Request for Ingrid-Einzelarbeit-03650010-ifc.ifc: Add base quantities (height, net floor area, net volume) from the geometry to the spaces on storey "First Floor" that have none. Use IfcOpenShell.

First a look at what the model holds.

```python
import ifcopenshell
import ifcopenshell.util.element
import ifcopenshell.util.unit

model = ifcopenshell.open("Ingrid-Einzelarbeit-03650010-ifc.ifc")
print(model.schema)
for unit_type in ("LENGTHUNIT", "AREAUNIT", "VOLUMEUNIT"):
    print(unit_type, ifcopenshell.util.unit.calculate_unit_scale(model, unit_type))
storey = next(s for s in model.by_type("IfcBuildingStorey") if s.Name == "First Floor")
spaces = [e for e in ifcopenshell.util.element.get_decomposition(storey) if e.is_a("IfcSpace")]
for e in sorted(spaces, key=lambda e: e.id()):
    print(e.id(), e.is_a(), e.Name, list(ifcopenshell.util.element.get_psets(e, qtos_only=True)), sep=" | ")
```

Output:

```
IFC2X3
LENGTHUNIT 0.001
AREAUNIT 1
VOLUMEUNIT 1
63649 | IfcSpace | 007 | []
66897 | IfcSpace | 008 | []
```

```python
import ifcopenshell
import ifcopenshell.api.pset
import ifcopenshell.geom
import ifcopenshell.util.element
import ifcopenshell.util.shape
import ifcopenshell.util.unit

model = ifcopenshell.open("Ingrid-Einzelarbeit-03650010-ifc.ifc")
unit_scale = ifcopenshell.util.unit.calculate_unit_scale(model)
area_scale = ifcopenshell.util.unit.calculate_unit_scale(model, "AREAUNIT")
volume_scale = ifcopenshell.util.unit.calculate_unit_scale(model, "VOLUMEUNIT")
settings = ifcopenshell.geom.settings()

storey = next(s for s in model.by_type("IfcBuildingStorey") if s.Name == "First Floor")
spaces = [e for e in ifcopenshell.util.element.get_decomposition(storey) if e.is_a("IfcSpace")]

for e in sorted(spaces, key=lambda e: e.id()):
    if ifcopenshell.util.element.get_psets(e, qtos_only=True, should_inherit=False):
        continue
    # Geometry comes back in metres, in the element's own axes.
    shape = ifcopenshell.geom.create_shape(settings, e)
    values = {
        "Height": ifcopenshell.util.shape.get_z(shape.geometry) / unit_scale,
        "NetFloorArea": ifcopenshell.util.shape.get_footprint_area(shape.geometry) / area_scale,
        "NetVolume": ifcopenshell.util.shape.get_volume(shape.geometry) / volume_scale,
    }
    qto = ifcopenshell.api.pset.add_qto(model, product=e, name="BaseQuantities")
    ifcopenshell.api.pset.edit_qto(model, qto=qto, properties=values)
    print(e.id(), {k: round(v, 3) for k, v in values.items()})

model.write("Ingrid-Einzelarbeit-03650010-ifc_edited.ifc")
```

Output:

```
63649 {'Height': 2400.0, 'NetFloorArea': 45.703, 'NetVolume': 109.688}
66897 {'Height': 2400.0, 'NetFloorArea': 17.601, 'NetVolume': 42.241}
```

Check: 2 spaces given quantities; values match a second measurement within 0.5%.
